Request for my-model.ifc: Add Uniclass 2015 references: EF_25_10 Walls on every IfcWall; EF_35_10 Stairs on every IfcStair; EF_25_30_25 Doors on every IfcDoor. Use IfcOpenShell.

First a look at what the model holds.

```python
import ifcopenshell

model = ifcopenshell.open("my-model.ifc")
print(model.schema)
print("classifications:", [c.Name for c in model.by_type("IfcClassification")])
for ifc_class in ("IfcDoor", "IfcRoof", "IfcStair", "IfcWall", "IfcWindow"):
    print(ifc_class, len(model.by_type(ifc_class)))
```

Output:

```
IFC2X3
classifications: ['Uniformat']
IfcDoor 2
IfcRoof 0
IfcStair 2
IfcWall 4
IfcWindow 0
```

```python
import ifcopenshell
import ifcopenshell.api.classification

model = ifcopenshell.open("my-model.ifc")

# IFC2X3 requires Source and Edition and has no link from the project to the system.
system = model.create_entity("IfcClassification", Source="NBS", Edition="2015", Name="Uniclass 2015")

codes = {
    "IfcWall": ("EF_25_10", "Walls"),
    "IfcStair": ("EF_35_10", "Stairs"),
    "IfcDoor": ("EF_25_30_25", "Doors"),
}
for ifc_class, (code, name) in codes.items():
    products = model.by_type(ifc_class)
    ifcopenshell.api.classification.add_reference(
        model, products=products, classification=system, identification=code, name=name
    )
    print(code, len(products))

model.write("my-model_rev.ifc")
```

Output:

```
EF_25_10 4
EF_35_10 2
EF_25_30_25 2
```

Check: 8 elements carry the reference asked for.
